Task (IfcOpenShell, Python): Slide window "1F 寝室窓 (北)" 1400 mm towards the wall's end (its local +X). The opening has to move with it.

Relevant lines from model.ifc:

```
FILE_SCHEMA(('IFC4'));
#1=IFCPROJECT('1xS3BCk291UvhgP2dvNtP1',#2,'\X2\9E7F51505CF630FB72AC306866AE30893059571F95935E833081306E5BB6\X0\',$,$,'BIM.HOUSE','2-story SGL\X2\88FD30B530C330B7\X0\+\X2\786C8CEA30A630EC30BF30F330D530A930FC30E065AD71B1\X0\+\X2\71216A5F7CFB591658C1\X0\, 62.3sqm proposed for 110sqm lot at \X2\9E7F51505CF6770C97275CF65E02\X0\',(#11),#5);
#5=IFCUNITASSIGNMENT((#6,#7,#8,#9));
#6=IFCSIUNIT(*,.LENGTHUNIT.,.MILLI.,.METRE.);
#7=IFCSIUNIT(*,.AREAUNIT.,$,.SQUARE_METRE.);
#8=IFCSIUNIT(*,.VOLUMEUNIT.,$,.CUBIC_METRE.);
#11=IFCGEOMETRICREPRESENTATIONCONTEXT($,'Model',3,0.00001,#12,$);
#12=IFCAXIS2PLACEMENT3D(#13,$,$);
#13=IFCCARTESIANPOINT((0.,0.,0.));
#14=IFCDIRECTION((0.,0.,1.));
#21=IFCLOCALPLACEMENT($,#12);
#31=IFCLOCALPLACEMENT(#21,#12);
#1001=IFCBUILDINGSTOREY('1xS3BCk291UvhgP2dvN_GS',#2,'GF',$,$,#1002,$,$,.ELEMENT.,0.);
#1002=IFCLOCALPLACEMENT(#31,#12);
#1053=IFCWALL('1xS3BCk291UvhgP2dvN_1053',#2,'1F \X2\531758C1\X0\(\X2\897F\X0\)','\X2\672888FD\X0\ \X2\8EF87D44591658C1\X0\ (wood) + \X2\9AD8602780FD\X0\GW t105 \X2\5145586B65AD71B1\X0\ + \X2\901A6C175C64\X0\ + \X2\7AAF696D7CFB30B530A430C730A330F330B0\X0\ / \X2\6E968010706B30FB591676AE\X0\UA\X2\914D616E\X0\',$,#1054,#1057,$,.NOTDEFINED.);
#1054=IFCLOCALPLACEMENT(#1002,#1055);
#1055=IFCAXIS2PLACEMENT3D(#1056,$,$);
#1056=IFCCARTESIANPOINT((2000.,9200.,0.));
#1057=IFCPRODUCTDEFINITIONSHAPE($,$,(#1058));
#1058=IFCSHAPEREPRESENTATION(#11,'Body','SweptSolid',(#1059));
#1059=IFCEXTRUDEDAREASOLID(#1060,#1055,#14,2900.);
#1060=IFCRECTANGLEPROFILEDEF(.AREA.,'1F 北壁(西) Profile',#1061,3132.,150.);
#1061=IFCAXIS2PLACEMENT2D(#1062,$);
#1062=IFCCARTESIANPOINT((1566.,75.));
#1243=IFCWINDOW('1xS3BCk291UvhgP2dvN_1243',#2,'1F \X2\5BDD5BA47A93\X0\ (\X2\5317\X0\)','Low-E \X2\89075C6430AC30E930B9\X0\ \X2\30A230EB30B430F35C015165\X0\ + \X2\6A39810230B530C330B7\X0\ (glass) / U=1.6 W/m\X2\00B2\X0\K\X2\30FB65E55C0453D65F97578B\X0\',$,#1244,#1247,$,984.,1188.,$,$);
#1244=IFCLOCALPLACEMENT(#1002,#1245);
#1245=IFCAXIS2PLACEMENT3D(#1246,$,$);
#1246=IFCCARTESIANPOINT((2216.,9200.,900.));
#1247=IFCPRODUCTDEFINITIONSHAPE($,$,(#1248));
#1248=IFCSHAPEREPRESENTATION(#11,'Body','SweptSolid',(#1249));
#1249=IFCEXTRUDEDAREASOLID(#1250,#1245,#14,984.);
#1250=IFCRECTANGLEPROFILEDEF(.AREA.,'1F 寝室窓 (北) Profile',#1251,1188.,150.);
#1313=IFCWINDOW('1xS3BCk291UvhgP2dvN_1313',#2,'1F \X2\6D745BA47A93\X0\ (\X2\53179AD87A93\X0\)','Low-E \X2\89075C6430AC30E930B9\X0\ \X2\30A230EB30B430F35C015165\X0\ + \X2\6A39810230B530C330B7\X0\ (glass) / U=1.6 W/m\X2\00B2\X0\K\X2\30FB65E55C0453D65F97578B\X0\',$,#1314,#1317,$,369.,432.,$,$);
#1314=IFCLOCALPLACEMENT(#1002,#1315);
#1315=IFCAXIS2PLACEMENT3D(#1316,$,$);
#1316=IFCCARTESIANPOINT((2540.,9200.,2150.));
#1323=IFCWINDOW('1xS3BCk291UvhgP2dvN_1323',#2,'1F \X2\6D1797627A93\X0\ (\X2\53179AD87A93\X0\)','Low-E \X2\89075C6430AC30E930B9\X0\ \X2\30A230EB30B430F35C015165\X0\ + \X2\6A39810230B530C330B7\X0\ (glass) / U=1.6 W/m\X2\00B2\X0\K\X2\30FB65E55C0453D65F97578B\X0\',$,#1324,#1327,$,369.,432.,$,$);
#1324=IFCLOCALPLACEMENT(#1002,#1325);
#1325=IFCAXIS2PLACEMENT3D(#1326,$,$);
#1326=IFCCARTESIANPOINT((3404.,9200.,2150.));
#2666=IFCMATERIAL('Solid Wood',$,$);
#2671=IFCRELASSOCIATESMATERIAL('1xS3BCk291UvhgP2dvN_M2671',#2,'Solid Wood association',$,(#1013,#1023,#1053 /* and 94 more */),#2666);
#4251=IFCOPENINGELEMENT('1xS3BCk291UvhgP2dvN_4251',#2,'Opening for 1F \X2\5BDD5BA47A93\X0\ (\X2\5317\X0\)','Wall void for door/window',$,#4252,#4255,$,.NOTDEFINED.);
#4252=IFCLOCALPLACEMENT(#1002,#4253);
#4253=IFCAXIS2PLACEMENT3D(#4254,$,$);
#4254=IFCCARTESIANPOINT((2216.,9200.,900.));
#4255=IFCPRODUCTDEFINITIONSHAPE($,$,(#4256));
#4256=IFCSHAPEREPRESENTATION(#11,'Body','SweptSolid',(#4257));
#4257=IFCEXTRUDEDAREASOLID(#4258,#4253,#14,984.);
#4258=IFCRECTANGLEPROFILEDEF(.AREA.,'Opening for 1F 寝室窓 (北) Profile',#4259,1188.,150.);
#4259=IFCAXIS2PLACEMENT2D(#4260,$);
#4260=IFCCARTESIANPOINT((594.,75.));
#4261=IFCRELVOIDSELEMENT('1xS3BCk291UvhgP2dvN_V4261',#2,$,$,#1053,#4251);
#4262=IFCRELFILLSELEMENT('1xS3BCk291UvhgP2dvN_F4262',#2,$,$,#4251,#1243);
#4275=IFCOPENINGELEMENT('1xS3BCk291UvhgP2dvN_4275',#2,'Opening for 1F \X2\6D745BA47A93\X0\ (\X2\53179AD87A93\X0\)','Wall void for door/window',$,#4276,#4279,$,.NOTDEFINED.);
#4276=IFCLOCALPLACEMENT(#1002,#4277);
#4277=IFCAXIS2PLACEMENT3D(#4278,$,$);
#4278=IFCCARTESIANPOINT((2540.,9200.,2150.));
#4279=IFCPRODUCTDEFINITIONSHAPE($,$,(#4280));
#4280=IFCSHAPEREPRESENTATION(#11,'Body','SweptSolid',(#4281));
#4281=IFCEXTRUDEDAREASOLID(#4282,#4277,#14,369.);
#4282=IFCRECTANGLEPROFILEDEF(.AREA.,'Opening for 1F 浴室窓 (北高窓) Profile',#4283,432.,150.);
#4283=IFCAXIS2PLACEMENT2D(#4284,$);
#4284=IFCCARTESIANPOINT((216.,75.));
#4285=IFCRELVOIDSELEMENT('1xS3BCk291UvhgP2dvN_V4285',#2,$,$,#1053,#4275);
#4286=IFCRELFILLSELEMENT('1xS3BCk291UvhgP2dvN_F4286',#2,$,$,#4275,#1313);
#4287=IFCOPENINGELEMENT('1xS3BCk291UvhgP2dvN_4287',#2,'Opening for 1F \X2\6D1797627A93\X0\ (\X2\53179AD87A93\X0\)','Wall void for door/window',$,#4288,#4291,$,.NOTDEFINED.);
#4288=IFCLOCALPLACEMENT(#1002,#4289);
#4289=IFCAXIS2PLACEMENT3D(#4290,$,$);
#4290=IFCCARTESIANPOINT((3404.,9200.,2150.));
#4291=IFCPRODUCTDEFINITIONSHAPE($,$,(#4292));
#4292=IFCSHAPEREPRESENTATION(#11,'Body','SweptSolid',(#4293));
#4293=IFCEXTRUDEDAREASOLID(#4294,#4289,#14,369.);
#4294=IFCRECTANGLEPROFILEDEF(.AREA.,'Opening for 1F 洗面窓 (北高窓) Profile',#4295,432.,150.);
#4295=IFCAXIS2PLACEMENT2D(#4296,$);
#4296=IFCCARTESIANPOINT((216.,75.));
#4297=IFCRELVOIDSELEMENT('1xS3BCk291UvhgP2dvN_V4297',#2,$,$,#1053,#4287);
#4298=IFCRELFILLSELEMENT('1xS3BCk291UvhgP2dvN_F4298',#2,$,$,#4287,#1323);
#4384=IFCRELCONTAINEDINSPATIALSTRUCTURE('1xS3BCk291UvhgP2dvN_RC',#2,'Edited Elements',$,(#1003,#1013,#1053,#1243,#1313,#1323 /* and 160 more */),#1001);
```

```python
import ifcopenshell
import ifcopenshell.api.geometry
import ifcopenshell.util.placement

model = ifcopenshell.open("model.ifc")

window = model.by_guid("1xS3BCk291UvhgP2dvN_1243")
opening = window.FillsVoids[0].RelatingOpeningElement
wall = opening.VoidsElements[0].RelatingBuildingElement

wall_matrix = ifcopenshell.util.placement.get_local_placement(wall.ObjectPlacement)
shift = wall_matrix[:3, 0] * 1400.0
before = ifcopenshell.util.placement.get_local_placement(window.ObjectPlacement)[:3, 3].copy()

# The window is not placed relative to its opening, so move both.
for product in (opening, window):
    matrix = ifcopenshell.util.placement.get_local_placement(product.ObjectPlacement)
    matrix[:3, 3] += shift
    ifcopenshell.api.geometry.edit_object_placement(model, product=product, matrix=matrix, is_si=False)

after = ifcopenshell.util.placement.get_local_placement(window.ObjectPlacement)[:3, 3]
print("window moved by", (after - before).round(3) + 0.0)

model.write("model-out.ifc")
```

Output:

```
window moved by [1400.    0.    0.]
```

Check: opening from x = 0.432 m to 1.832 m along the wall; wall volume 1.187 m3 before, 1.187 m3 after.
